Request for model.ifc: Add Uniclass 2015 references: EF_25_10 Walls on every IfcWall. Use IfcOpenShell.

First a look at what the model holds.

```python
import ifcopenshell

model = ifcopenshell.open("model.ifc")
print(model.schema)
print("classifications:", [c.Name for c in model.by_type("IfcClassification")])
for ifc_class in ("IfcDoor", "IfcRoof", "IfcStair", "IfcWall", "IfcWindow"):
    print(ifc_class, len(model.by_type(ifc_class)))
```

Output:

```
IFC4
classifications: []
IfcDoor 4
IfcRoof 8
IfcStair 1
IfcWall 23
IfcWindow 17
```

```python
import ifcopenshell
import ifcopenshell.api.classification

model = ifcopenshell.open("model.ifc")

system = ifcopenshell.api.classification.add_classification(model, classification="Uniclass 2015")

codes = {
    "IfcWall": ("EF_25_10", "Walls"),
}
for ifc_class, (code, name) in codes.items():
    products = model.by_type(ifc_class)
    ifcopenshell.api.classification.add_reference(
        model, products=products, classification=system, identification=code, name=name
    )
    print(code, len(products))

model.write("model_edited.ifc")
```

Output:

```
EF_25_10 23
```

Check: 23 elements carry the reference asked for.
